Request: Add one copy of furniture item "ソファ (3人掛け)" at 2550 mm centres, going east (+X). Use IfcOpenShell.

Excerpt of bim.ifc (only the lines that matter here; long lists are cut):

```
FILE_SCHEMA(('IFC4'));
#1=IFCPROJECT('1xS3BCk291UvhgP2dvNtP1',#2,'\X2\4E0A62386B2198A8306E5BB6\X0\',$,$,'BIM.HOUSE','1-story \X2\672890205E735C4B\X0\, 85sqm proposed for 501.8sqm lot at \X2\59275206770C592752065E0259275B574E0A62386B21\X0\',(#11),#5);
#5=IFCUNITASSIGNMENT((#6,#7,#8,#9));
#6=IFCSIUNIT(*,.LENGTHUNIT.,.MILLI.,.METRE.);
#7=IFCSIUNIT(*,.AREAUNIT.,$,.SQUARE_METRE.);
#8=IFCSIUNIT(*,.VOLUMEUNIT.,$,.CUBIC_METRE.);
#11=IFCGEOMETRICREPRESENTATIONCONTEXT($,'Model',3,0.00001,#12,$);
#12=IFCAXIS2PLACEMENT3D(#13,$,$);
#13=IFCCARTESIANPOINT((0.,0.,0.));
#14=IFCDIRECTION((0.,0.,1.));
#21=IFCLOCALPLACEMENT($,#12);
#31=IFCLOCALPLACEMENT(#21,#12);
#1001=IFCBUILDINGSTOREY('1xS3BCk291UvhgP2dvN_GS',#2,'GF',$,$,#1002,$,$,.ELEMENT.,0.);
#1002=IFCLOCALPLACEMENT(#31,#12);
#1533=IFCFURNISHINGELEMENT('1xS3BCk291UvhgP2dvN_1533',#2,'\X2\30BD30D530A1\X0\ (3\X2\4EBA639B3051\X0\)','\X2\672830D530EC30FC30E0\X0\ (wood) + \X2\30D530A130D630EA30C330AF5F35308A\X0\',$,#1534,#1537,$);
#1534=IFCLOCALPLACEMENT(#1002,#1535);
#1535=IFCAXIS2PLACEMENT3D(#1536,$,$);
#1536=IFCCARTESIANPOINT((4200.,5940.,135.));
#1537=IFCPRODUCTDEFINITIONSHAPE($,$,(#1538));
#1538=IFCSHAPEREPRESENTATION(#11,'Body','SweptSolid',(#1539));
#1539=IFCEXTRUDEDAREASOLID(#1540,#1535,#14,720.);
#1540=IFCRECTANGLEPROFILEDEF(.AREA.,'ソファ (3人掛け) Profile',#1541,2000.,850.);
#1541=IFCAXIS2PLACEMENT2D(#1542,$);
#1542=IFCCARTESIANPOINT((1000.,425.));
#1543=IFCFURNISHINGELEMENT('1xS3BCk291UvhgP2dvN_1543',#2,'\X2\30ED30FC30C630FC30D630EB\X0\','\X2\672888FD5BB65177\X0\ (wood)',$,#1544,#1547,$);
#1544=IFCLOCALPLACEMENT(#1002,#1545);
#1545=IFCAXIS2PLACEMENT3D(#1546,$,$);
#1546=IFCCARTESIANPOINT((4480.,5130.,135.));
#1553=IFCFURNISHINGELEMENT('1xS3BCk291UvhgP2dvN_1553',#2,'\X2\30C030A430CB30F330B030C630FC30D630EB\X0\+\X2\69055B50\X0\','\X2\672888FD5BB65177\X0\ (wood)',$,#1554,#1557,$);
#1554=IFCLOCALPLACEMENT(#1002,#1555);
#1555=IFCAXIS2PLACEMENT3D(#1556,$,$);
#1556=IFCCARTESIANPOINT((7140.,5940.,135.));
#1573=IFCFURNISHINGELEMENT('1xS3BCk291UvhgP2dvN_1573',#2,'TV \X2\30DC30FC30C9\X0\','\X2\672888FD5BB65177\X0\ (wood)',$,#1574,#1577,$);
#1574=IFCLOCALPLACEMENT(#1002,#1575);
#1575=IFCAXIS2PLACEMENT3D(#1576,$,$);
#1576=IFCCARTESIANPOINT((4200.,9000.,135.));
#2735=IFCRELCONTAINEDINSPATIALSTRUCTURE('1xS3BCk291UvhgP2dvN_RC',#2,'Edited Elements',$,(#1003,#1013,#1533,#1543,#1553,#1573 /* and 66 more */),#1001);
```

```python
import numpy as np
import ifcopenshell
import ifcopenshell.api.geometry
import ifcopenshell.api.root
import ifcopenshell.util.element
import ifcopenshell.util.placement
import ifcopenshell.util.unit

model = ifcopenshell.open("bim.ifc")
unit_scale = ifcopenshell.util.unit.calculate_unit_scale(model)


def reuse_history(source, copy):
    """copy_class also copies each property set's owner history, people and application; keep the originals."""
    for rel in copy.IsDefinedBy:
        if rel.is_a("IfcRelDefinesByProperties") and (history := rel.RelatingPropertyDefinition.OwnerHistory):
            rel.RelatingPropertyDefinition.OwnerHistory = source.OwnerHistory
            ifcopenshell.util.element.remove_deep2(model, history)


source = model.by_id(1533)
base = ifcopenshell.util.placement.get_local_placement(source.ObjectPlacement)
step = np.array([1.0, 0.0, 0.0]) * 2.55 / unit_scale

for i in range(1, 2):
    copy = ifcopenshell.api.root.copy_class(model, product=source)
    copy.Representation = ifcopenshell.util.element.copy_deep(
        model, source.Representation, exclude=["IfcGeometricRepresentationContext", "IfcRepresentationMap"]
    )
    reuse_history(source, copy)
    matrix = base.copy()
    matrix[:3, 3] += i * step
    print("added at", matrix[:3, 3].round(3) + 0.0)
    ifcopenshell.api.geometry.edit_object_placement(model, product=copy, matrix=matrix, is_si=False)

model.write("bim_updated.ifc")
```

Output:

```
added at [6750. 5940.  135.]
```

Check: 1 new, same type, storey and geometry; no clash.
